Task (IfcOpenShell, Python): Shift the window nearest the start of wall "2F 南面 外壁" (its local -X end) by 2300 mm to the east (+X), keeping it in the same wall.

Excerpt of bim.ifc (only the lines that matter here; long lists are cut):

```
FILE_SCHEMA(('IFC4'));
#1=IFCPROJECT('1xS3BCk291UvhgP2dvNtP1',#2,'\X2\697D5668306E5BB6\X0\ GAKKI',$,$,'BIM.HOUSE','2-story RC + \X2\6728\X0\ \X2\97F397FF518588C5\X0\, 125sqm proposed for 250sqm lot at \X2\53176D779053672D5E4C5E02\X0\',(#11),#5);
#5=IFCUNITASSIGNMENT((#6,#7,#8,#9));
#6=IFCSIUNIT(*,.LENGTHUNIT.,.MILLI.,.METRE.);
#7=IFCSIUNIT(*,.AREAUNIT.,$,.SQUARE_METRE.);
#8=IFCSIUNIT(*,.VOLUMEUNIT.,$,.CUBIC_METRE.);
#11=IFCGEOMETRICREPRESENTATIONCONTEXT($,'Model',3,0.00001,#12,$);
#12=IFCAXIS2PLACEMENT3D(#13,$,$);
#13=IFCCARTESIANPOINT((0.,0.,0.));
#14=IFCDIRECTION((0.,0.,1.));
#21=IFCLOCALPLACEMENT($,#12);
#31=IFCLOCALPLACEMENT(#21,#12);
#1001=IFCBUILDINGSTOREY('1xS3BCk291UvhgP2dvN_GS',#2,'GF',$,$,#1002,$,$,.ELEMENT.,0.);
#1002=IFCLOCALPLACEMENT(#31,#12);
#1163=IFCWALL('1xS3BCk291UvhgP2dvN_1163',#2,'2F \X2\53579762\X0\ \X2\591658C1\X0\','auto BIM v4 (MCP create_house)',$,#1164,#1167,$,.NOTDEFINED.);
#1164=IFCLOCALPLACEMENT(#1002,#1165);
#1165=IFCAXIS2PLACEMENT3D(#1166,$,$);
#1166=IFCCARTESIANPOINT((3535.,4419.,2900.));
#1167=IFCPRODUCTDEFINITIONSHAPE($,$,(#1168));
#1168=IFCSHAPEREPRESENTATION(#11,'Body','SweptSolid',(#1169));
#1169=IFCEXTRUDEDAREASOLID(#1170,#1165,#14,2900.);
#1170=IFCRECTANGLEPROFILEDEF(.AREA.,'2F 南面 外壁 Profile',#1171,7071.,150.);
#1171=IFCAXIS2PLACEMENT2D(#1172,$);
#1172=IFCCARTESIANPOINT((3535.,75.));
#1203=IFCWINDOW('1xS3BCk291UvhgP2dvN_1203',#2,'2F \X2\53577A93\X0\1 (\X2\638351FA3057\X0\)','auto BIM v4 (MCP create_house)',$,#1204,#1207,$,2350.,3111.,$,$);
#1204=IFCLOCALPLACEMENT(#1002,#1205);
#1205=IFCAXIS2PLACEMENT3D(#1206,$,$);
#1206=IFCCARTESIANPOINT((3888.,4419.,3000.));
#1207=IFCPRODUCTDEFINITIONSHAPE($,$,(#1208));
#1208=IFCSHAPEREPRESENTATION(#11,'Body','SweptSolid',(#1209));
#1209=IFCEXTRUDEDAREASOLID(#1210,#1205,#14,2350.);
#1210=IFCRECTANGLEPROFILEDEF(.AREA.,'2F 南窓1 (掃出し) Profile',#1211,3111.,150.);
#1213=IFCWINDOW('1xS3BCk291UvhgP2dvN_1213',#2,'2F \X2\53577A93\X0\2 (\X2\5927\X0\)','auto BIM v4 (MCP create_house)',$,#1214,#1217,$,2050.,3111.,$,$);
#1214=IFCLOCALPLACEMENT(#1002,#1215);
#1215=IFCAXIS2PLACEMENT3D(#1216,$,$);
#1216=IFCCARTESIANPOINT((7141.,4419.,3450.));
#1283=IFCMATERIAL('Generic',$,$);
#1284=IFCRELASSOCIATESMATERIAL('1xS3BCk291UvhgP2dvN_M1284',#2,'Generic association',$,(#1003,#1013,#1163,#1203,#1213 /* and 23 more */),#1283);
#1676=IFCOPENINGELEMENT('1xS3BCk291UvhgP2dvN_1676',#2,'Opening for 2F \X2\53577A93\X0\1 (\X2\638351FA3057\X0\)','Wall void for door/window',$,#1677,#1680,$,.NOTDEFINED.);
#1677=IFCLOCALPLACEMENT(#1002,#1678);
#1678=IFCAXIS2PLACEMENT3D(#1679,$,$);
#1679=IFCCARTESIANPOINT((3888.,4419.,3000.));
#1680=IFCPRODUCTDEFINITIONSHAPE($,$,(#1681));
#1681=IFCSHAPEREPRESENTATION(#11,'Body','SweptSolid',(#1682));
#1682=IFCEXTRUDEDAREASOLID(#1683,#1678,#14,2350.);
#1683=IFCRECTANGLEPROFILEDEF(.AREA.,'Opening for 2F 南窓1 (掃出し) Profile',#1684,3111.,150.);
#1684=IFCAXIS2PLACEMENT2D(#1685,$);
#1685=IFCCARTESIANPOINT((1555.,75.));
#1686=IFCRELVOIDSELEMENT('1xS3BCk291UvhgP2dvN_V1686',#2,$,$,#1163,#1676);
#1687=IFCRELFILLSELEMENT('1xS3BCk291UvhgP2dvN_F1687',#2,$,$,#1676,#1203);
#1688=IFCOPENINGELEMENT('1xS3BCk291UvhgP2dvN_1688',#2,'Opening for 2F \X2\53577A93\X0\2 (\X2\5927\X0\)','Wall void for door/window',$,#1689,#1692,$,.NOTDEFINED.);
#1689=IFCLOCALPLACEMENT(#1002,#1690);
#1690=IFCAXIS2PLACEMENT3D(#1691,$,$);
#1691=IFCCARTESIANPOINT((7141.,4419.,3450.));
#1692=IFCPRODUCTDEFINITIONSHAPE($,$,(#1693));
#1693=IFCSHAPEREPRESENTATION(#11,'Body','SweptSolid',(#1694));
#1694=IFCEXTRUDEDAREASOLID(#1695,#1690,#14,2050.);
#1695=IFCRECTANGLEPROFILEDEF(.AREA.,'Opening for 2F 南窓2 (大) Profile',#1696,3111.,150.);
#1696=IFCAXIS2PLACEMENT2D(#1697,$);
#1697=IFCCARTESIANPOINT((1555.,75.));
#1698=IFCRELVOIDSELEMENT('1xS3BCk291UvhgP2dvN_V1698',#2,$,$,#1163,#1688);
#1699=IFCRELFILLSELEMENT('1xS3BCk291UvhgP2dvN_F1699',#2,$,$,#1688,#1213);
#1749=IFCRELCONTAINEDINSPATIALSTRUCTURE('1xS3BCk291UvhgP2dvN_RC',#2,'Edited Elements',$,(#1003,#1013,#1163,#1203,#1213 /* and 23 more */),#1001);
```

```python
import ifcopenshell
import ifcopenshell.api.geometry
import ifcopenshell.util.placement

model = ifcopenshell.open("bim.ifc")

window = model.by_guid("1xS3BCk291UvhgP2dvN_1203")
opening = window.FillsVoids[0].RelatingOpeningElement
wall = opening.VoidsElements[0].RelatingBuildingElement

wall_matrix = ifcopenshell.util.placement.get_local_placement(wall.ObjectPlacement)
shift = wall_matrix[:3, 0] * 2300.0
before = ifcopenshell.util.placement.get_local_placement(window.ObjectPlacement)[:3, 3].copy()

# The window is not placed relative to its opening, so move both.
for product in (opening, window):
    matrix = ifcopenshell.util.placement.get_local_placement(product.ObjectPlacement)
    matrix[:3, 3] += shift
    ifcopenshell.api.geometry.edit_object_placement(model, product=product, matrix=matrix, is_si=False)

after = ifcopenshell.util.placement.get_local_placement(window.ObjectPlacement)[:3, 3]
print("window moved by", (after - before).round(3) + 0.0)

model.write("bim_edited.ifc")
```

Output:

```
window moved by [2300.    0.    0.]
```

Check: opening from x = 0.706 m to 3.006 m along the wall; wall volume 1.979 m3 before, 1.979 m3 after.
